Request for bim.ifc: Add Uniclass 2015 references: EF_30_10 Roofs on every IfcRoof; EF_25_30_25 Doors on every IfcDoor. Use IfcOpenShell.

First a look at what the model holds.

```python
import ifcopenshell

model = ifcopenshell.open("bim.ifc")
print(model.schema)
print("classifications:", [c.Name for c in model.by_type("IfcClassification")])
for ifc_class in ("IfcDoor", "IfcRoof", "IfcStair", "IfcWall", "IfcWindow"):
    print(ifc_class, len(model.by_type(ifc_class)))
```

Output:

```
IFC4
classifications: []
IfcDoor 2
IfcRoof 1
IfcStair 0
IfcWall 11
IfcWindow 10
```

```python
import ifcopenshell
import ifcopenshell.api.classification

model = ifcopenshell.open("bim.ifc")

system = ifcopenshell.api.classification.add_classification(model, classification="Uniclass 2015")

codes = {
    "IfcRoof": ("EF_30_10", "Roofs"),
    "IfcDoor": ("EF_25_30_25", "Doors"),
}
for ifc_class, (code, name) in codes.items():
    products = model.by_type(ifc_class)
    ifcopenshell.api.classification.add_reference(
        model, products=products, classification=system, identification=code, name=name
    )
    print(code, len(products))

model.write("bim_rev.ifc")
```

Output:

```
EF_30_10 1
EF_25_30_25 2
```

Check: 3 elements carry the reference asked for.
